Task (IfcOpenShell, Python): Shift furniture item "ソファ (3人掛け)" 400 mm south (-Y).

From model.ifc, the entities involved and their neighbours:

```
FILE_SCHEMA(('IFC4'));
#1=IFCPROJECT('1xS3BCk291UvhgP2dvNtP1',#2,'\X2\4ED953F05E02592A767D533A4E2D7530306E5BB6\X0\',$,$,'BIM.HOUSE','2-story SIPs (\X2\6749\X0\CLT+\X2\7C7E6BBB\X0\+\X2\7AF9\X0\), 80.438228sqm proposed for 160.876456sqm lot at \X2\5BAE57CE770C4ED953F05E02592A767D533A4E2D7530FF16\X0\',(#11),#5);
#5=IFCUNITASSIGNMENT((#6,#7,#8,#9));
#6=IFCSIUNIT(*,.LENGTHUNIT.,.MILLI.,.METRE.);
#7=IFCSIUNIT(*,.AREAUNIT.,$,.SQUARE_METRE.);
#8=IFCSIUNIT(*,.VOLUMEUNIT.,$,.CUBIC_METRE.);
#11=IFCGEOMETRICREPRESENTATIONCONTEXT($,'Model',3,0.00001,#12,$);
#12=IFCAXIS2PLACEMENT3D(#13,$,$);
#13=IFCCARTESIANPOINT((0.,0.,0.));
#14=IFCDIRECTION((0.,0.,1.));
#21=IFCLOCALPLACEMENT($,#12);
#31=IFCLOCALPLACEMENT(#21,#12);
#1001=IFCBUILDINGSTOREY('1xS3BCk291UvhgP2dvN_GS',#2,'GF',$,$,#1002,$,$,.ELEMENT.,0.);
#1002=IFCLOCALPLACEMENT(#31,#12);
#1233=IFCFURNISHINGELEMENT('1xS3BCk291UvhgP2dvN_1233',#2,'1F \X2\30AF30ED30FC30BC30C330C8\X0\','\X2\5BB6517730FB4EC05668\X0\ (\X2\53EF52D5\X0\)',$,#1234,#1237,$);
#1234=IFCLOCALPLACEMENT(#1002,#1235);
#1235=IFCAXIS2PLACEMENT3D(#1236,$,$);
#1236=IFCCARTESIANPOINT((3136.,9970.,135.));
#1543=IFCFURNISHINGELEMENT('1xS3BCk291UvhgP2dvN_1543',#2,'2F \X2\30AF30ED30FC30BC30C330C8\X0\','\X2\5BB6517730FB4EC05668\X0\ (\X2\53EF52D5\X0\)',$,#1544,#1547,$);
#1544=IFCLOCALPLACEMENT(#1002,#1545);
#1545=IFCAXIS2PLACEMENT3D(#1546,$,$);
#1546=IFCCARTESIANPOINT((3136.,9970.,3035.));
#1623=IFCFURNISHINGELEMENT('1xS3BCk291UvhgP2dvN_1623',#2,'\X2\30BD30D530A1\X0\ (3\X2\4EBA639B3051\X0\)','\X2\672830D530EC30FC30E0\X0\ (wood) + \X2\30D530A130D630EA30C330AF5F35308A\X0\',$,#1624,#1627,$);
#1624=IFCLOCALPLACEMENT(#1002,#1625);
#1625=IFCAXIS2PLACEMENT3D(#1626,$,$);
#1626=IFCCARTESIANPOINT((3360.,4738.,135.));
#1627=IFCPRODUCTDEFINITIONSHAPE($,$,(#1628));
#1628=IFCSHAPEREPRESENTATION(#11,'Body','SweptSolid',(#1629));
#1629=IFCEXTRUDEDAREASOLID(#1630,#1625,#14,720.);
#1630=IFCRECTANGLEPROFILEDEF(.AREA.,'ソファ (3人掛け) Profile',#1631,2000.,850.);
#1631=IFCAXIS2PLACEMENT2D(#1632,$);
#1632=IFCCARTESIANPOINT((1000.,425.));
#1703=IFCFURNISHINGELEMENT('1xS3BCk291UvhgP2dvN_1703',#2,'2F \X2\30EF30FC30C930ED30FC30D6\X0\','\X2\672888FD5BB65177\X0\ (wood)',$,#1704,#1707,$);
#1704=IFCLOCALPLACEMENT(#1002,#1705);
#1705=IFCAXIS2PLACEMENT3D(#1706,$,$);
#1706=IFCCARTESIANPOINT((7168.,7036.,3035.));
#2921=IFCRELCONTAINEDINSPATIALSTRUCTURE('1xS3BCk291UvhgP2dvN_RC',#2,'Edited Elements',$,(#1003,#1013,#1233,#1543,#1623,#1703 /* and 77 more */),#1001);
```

```python
import ifcopenshell
import ifcopenshell.api.geometry
import ifcopenshell.util.placement
import ifcopenshell.util.unit

model = ifcopenshell.open("model.ifc")
unit_scale = ifcopenshell.util.unit.calculate_unit_scale(model)

item = model.by_id(1623)
matrix = ifcopenshell.util.placement.get_local_placement(item.ObjectPlacement)
matrix[1, 3] -= 0.4 / unit_scale
ifcopenshell.api.geometry.edit_object_placement(model, product=item, matrix=matrix, is_si=False)

print(ifcopenshell.util.placement.get_local_placement(item.ObjectPlacement).round(3) + 0.0)

model.write("model_v2.ifc")
```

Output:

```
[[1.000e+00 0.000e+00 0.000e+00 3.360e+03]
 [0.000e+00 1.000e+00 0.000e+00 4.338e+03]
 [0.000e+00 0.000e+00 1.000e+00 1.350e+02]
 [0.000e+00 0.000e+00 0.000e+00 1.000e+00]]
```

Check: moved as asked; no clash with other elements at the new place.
